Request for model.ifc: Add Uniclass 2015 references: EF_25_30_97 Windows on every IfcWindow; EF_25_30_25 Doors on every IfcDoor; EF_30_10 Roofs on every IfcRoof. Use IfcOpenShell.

First a look at what the model holds.

```python
import ifcopenshell

model = ifcopenshell.open("model.ifc")
print(model.schema)
print("classifications:", [c.Name for c in model.by_type("IfcClassification")])
for ifc_class in ("IfcDoor", "IfcRoof", "IfcStair", "IfcWall", "IfcWindow"):
    print(ifc_class, len(model.by_type(ifc_class)))
```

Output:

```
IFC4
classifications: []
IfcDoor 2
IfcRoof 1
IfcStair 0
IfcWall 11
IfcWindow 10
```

```python
import ifcopenshell
import ifcopenshell.api.classification

model = ifcopenshell.open("model.ifc")

system = ifcopenshell.api.classification.add_classification(model, classification="Uniclass 2015")

codes = {
    "IfcWindow": ("EF_25_30_97", "Windows"),
    "IfcDoor": ("EF_25_30_25", "Doors"),
    "IfcRoof": ("EF_30_10", "Roofs"),
}
for ifc_class, (code, name) in codes.items():
    products = model.by_type(ifc_class)
    ifcopenshell.api.classification.add_reference(
        model, products=products, classification=system, identification=code, name=name
    )
    print(code, len(products))

model.write("model-out.ifc")
```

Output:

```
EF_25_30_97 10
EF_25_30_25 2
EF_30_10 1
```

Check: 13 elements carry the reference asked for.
